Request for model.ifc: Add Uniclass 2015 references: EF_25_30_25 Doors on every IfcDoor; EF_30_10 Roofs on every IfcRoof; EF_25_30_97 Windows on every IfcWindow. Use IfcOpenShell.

First a look at what the model holds.

```python
import ifcopenshell

model = ifcopenshell.open("model.ifc")
print(model.schema)
print("classifications:", [c.Name for c in model.by_type("IfcClassification")])
for ifc_class in ("IfcDoor", "IfcRoof", "IfcStair", "IfcWall", "IfcWindow"):
    print(ifc_class, len(model.by_type(ifc_class)))
```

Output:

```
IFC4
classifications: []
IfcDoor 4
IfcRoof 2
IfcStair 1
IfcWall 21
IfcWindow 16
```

```python
import ifcopenshell
import ifcopenshell.api.classification

model = ifcopenshell.open("model.ifc")

system = ifcopenshell.api.classification.add_classification(model, classification="Uniclass 2015")

codes = {
    "IfcDoor": ("EF_25_30_25", "Doors"),
    "IfcRoof": ("EF_30_10", "Roofs"),
    "IfcWindow": ("EF_25_30_97", "Windows"),
}
for ifc_class, (code, name) in codes.items():
    products = model.by_type(ifc_class)
    ifcopenshell.api.classification.add_reference(
        model, products=products, classification=system, identification=code, name=name
    )
    print(code, len(products))

model.write("model-out.ifc")
```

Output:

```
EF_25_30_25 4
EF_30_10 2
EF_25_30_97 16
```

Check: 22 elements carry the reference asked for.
